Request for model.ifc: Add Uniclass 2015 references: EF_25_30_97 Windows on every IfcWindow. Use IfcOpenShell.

First a look at what the model holds.

```python
import ifcopenshell

model = ifcopenshell.open("model.ifc")
print(model.schema)
print("classifications:", [c.Name for c in model.by_type("IfcClassification")])
for ifc_class in ("IfcDoor", "IfcRoof", "IfcStair", "IfcWall", "IfcWindow"):
    print(ifc_class, len(model.by_type(ifc_class)))
```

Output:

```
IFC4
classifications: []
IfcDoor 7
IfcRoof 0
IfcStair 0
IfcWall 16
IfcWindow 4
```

```python
import ifcopenshell
import ifcopenshell.api.classification

model = ifcopenshell.open("model.ifc")

system = ifcopenshell.api.classification.add_classification(model, classification="Uniclass 2015")

codes = {
    "IfcWindow": ("EF_25_30_97", "Windows"),
}
for ifc_class, (code, name) in codes.items():
    products = model.by_type(ifc_class)
    ifcopenshell.api.classification.add_reference(
        model, products=products, classification=system, identification=code, name=name
    )
    print(code, len(products))

model.write("model_updated.ifc")
```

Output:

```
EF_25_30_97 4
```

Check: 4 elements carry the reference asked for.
